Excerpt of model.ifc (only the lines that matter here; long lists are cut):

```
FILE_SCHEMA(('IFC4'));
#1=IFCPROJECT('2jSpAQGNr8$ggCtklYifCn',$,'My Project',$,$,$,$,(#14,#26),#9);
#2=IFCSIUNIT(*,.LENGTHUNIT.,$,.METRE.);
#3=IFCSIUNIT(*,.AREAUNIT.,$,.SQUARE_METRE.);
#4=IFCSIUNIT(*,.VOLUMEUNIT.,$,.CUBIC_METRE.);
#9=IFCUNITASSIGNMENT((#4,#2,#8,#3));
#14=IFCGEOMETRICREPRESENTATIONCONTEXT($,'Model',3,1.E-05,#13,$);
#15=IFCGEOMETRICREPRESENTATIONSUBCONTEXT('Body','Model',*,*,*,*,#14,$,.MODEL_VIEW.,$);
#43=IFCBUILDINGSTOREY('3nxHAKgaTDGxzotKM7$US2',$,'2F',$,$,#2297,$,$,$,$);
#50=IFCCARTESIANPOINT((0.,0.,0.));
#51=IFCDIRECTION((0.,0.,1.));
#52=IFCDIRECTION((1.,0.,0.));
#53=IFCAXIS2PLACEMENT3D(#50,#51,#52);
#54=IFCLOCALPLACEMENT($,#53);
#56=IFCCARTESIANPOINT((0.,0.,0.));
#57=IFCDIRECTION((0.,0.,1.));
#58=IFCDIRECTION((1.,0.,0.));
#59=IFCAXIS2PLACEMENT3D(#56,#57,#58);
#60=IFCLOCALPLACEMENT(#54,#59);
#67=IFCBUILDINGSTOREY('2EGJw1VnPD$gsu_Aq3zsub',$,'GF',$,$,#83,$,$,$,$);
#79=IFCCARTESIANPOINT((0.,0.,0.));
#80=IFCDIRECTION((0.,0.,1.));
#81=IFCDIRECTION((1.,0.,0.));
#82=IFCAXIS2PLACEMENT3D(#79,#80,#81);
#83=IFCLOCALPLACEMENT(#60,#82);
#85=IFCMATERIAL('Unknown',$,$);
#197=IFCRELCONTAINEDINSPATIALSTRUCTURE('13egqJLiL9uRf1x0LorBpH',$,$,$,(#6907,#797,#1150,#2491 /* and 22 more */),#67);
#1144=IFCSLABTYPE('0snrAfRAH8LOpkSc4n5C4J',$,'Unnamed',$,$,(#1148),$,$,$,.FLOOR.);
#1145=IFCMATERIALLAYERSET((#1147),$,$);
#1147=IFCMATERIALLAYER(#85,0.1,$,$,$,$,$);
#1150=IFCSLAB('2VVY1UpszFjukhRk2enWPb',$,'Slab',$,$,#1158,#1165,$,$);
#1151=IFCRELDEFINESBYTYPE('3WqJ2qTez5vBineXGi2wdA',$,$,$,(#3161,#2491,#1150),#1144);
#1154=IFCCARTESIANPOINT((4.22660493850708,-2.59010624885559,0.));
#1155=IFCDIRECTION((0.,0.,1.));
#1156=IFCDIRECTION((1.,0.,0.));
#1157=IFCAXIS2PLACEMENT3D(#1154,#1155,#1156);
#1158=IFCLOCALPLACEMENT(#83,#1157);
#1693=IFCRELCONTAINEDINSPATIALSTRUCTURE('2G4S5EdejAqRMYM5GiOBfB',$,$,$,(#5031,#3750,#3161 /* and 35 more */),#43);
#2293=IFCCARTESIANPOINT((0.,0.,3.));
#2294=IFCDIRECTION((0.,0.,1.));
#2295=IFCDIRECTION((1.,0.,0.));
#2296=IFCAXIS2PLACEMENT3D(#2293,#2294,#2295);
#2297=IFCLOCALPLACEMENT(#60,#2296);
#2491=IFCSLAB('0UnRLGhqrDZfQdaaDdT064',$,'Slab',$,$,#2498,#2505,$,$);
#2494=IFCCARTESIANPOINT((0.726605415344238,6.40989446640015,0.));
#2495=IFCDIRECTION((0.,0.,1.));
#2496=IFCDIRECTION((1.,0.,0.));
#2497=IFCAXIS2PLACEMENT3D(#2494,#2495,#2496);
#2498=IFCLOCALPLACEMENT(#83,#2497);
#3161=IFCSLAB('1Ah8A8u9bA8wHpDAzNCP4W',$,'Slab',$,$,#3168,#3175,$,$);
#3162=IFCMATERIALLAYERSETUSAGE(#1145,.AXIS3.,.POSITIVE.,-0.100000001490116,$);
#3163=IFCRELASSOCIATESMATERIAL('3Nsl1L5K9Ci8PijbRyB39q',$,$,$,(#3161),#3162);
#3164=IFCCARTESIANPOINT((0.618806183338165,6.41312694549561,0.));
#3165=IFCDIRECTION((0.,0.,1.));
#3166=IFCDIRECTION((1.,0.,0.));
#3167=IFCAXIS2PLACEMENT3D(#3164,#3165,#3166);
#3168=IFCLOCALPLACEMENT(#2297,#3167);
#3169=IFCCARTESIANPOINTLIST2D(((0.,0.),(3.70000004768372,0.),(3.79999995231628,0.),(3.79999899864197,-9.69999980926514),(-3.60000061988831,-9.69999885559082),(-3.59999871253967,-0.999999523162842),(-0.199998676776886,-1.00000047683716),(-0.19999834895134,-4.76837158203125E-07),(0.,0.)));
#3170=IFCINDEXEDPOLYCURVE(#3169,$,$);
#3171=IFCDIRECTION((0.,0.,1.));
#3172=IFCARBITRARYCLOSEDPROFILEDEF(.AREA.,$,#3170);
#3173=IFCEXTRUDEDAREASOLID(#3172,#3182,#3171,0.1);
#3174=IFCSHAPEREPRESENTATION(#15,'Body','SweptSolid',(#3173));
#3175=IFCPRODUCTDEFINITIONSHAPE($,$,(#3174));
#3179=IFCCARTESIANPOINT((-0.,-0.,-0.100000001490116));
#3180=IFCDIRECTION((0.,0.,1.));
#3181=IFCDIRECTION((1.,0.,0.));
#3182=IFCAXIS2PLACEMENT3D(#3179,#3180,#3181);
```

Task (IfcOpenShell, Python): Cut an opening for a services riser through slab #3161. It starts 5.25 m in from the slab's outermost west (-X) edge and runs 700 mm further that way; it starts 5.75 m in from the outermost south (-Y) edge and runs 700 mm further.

```python
import numpy as np
import ifcopenshell
import ifcopenshell.api.feature
import ifcopenshell.api.geometry
import ifcopenshell.api.root
import ifcopenshell.geom
import ifcopenshell.util.placement
import ifcopenshell.util.representation
import ifcopenshell.util.shape
import ifcopenshell.util.unit

model = ifcopenshell.open("model.ifc")
unit_scale = ifcopenshell.util.unit.calculate_unit_scale(model)
settings = ifcopenshell.geom.settings()


def volume(element):
    """Net volume in cubic metres, openings subtracted."""
    shape = ifcopenshell.geom.create_shape(settings, element)
    return ifcopenshell.util.shape.get_volume(shape.geometry)


slab = model.by_id(3161)
before = volume(slab)

# Extent in the slab's own axes, in metres. The edges named are its -X and -Y sides.
slab_shape = ifcopenshell.geom.create_shape(settings, slab)
vertices = ifcopenshell.util.shape.get_vertices(slab_shape.geometry)
x_min, y_min, bottom = vertices.min(axis=0)
top = vertices[:, 2].max()

opening = ifcopenshell.api.root.create_entity(model, ifc_class="IfcOpeningElement", name="Services riser opening", predefined_type="OPENING")
context = ifcopenshell.util.representation.get_context(model, "Model", "Body", "MODEL_VIEW")
width, depth = 0.7, 0.7
outline = [(0.0, 0.0), (width, 0.0), (width, depth), (0.0, depth), (0.0, 0.0)]
# Overshoot both faces by 50 mm so the cut is clean.
shape = ifcopenshell.api.geometry.add_slab_representation(
    model, context=context, depth=top - bottom + 0.1, polyline=outline
)
ifcopenshell.api.geometry.assign_representation(model, product=opening, representation=shape)

matrix = ifcopenshell.util.placement.get_local_placement(slab.ObjectPlacement)
matrix[:, 3] = matrix @ np.append(np.array([x_min + 5.25, y_min + 5.75, bottom - 0.05]) / unit_scale, 1.0)
ifcopenshell.api.geometry.edit_object_placement(model, product=opening, matrix=matrix, is_si=False)
ifcopenshell.api.feature.add_feature(model, feature=opening, element=slab)

after = volume(slab)

print(f"slab volume {before:.3f} -> {after:.3f} m3")

model.write("model_v2.ifc")
```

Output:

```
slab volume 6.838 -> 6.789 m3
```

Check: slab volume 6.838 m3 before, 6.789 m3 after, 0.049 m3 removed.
